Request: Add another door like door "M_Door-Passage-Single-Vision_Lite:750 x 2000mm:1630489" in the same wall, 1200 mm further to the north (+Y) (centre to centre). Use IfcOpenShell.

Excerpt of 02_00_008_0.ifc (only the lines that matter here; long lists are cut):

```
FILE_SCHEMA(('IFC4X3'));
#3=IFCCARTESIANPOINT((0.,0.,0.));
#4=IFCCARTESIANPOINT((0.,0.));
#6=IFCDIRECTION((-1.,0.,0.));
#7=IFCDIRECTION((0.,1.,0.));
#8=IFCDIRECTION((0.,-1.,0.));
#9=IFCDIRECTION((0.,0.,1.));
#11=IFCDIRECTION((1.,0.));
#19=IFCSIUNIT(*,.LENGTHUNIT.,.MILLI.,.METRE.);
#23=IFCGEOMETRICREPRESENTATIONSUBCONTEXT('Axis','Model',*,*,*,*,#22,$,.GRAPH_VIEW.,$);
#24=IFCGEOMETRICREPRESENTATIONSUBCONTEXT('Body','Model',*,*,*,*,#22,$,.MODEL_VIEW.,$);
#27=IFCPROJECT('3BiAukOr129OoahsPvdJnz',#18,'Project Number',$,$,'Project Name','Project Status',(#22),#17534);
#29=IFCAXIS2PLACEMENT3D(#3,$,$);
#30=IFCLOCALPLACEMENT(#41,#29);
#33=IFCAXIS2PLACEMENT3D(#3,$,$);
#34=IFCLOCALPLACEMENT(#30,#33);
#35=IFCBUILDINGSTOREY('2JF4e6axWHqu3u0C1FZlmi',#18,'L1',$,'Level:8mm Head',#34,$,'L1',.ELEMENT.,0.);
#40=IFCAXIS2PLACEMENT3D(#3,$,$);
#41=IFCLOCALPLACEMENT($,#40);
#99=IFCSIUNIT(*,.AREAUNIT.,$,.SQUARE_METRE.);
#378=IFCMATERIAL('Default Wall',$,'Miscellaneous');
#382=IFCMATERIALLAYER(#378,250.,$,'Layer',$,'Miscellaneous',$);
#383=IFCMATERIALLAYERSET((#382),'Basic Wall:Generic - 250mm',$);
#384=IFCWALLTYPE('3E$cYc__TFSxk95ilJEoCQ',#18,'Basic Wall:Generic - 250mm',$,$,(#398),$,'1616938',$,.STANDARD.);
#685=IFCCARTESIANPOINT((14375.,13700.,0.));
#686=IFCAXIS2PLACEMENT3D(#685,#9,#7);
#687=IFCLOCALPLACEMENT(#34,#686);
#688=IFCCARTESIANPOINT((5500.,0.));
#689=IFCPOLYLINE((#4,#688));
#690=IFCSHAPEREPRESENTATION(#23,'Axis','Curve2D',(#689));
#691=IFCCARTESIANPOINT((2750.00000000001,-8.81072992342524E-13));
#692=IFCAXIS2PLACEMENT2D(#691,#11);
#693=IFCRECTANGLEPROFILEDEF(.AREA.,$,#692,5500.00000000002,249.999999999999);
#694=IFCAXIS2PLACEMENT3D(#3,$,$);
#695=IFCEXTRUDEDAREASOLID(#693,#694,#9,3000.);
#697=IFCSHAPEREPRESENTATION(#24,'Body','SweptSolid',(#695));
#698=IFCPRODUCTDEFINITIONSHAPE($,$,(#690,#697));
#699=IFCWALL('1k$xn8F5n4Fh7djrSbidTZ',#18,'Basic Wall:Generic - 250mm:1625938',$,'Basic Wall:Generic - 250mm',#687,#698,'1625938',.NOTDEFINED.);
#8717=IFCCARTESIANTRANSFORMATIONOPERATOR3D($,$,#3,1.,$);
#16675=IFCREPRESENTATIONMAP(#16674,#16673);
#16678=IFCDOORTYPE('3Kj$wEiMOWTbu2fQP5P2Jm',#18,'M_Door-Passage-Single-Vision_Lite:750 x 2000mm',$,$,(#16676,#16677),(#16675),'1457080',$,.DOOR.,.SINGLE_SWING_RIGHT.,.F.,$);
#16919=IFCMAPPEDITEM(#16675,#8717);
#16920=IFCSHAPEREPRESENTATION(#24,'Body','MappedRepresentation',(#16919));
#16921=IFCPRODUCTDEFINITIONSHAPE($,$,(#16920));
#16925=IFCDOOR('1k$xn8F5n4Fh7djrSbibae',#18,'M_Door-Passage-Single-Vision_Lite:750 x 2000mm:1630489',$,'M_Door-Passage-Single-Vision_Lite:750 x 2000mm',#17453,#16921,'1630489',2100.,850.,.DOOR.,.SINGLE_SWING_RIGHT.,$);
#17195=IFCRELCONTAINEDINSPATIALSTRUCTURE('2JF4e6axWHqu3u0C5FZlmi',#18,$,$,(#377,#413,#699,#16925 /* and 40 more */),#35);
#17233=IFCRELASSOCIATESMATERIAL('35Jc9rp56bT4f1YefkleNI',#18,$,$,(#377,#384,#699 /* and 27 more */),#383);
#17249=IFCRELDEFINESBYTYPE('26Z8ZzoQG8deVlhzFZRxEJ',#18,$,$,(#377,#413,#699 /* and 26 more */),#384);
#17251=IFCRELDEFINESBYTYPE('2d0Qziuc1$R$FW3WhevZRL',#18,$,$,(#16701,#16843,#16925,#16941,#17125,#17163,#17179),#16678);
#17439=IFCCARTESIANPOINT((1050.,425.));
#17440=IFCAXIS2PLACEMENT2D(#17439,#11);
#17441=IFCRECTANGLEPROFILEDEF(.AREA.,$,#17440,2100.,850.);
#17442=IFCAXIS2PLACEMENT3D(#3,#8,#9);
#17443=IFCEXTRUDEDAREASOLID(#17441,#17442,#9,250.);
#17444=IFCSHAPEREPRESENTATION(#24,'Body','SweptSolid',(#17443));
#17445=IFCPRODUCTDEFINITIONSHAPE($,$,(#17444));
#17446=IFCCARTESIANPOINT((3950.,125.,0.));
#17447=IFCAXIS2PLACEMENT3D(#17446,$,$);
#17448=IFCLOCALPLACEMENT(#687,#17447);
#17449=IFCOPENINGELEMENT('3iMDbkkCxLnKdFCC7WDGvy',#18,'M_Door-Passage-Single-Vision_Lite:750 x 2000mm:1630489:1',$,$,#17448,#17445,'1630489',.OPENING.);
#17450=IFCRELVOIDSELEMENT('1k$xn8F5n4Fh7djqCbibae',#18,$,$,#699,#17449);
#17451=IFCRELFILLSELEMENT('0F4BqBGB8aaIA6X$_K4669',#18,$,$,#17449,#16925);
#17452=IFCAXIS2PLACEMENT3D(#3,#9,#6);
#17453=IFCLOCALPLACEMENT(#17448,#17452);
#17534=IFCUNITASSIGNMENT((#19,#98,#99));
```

```python
import ifcopenshell
import ifcopenshell.api.feature
import ifcopenshell.api.geometry
import ifcopenshell.api.root
import ifcopenshell.geom
import ifcopenshell.util.element
import ifcopenshell.util.placement
import ifcopenshell.util.shape

model = ifcopenshell.open("02_00_008_0.ifc")
settings = ifcopenshell.geom.settings()


def volume(element):
    """Net volume in cubic metres, openings subtracted."""
    shape = ifcopenshell.geom.create_shape(settings, element)
    return ifcopenshell.util.shape.get_volume(shape.geometry)


def reuse_history(source, copy):
    """copy_class also copies each property set's owner history, people and application; keep the originals."""
    for rel in copy.IsDefinedBy:
        if rel.is_a("IfcRelDefinesByProperties") and (history := rel.RelatingPropertyDefinition.OwnerHistory):
            rel.RelatingPropertyDefinition.OwnerHistory = source.OwnerHistory
            ifcopenshell.util.element.remove_deep2(model, history)


door = model.by_id(16925)
opening = door.FillsVoids[0].RelatingOpeningElement
wall = opening.VoidsElements[0].RelatingBuildingElement
before = volume(wall)
shift = ifcopenshell.util.placement.get_local_placement(wall.ObjectPlacement)[:3, 0] * 1200.0

# copy_class copies the void relationship, type, container and properties, but no geometry.
new_opening = ifcopenshell.api.root.copy_class(model, product=opening)
new_opening.Representation = ifcopenshell.util.element.copy_deep(
    model, opening.Representation, exclude=["IfcGeometricRepresentationContext", "IfcRepresentationMap"]
)
new_opening.Name = "M_Door-Passage-Single-Vision_Lite:750 x 2000mm"
new_opening.Tag = None
new_door = ifcopenshell.api.root.copy_class(model, product=door)
new_door.Representation = ifcopenshell.util.element.copy_deep(
    model, door.Representation, exclude=["IfcGeometricRepresentationContext", "IfcRepresentationMap"]
)
new_door.Name = "M_Door-Passage-Single-Vision_Lite:750 x 2000mm"
new_door.Tag = None
reuse_history(door, new_door)
ifcopenshell.api.feature.add_filling(model, opening=new_opening, element=new_door)

for old, new in ((opening, new_opening), (door, new_door)):
    matrix = ifcopenshell.util.placement.get_local_placement(old.ObjectPlacement)
    matrix[:3, 3] += shift
    ifcopenshell.api.geometry.edit_object_placement(model, product=new, matrix=matrix, is_si=False)

after = volume(wall)

print(f"wall volume {before:.3f} -> {after:.3f} m3")

model.write("02_00_008_0_edited.ifc")
```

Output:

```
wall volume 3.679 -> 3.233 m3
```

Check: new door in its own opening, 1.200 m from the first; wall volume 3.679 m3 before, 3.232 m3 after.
